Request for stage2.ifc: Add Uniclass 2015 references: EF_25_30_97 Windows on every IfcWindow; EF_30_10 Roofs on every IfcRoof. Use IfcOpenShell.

First a look at what the model holds.

```python
import ifcopenshell

model = ifcopenshell.open("stage2.ifc")
print(model.schema)
print("classifications:", [c.Name for c in model.by_type("IfcClassification")])
for ifc_class in ("IfcDoor", "IfcRoof", "IfcStair", "IfcWall", "IfcWindow"):
    print(ifc_class, len(model.by_type(ifc_class)))
```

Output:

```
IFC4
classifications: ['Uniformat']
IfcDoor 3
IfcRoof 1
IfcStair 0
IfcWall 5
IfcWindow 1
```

```python
import ifcopenshell
import ifcopenshell.api.classification

model = ifcopenshell.open("stage2.ifc")

system = ifcopenshell.api.classification.add_classification(model, classification="Uniclass 2015")

codes = {
    "IfcWindow": ("EF_25_30_97", "Windows"),
    "IfcRoof": ("EF_30_10", "Roofs"),
}
for ifc_class, (code, name) in codes.items():
    products = model.by_type(ifc_class)
    ifcopenshell.api.classification.add_reference(
        model, products=products, classification=system, identification=code, name=name
    )
    print(code, len(products))

model.write("stage2_edited.ifc")
```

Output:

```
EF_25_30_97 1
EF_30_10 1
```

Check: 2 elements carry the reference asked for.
